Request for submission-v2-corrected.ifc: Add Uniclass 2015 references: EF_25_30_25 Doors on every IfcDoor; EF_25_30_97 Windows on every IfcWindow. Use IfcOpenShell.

First a look at what the model holds.

```python
import ifcopenshell

model = ifcopenshell.open("submission-v2-corrected.ifc")
print(model.schema)
print("classifications:", [c.Name for c in model.by_type("IfcClassification")])
for ifc_class in ("IfcDoor", "IfcRoof", "IfcStair", "IfcWall", "IfcWindow"):
    print(ifc_class, len(model.by_type(ifc_class)))
```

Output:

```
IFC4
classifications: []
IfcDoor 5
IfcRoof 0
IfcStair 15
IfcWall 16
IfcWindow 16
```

```python
import ifcopenshell
import ifcopenshell.api.classification

model = ifcopenshell.open("submission-v2-corrected.ifc")

system = ifcopenshell.api.classification.add_classification(model, classification="Uniclass 2015")

codes = {
    "IfcDoor": ("EF_25_30_25", "Doors"),
    "IfcWindow": ("EF_25_30_97", "Windows"),
}
for ifc_class, (code, name) in codes.items():
    products = model.by_type(ifc_class)
    ifcopenshell.api.classification.add_reference(
        model, products=products, classification=system, identification=code, name=name
    )
    print(code, len(products))

model.write("submission-v2-corrected_updated.ifc")
```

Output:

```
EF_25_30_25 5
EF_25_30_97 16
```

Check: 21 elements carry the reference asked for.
